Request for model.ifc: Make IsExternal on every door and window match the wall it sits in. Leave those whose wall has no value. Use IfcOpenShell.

First a look at what the model holds.

```python
import ifcopenshell
import ifcopenshell.util.element

model = ifcopenshell.open("model.ifc")
print(model.schema)
seen = {}
for e in model.by_type("IfcDoor") + model.by_type("IfcWindow"):
    if not e.FillsVoids:
        continue
    host = e.FillsVoids[0].RelatingOpeningElement.VoidsElements[0].RelatingBuildingElement
    own = ifcopenshell.util.element.get_pset(e, f"Pset_{e.is_a()[3:].removesuffix('StandardCase')}Common", "IsExternal")
    wall = ifcopenshell.util.element.get_pset(host, "Pset_WallCommon", "IsExternal")
    seen[e.is_a(), own, wall] = seen.get((e.is_a(), own, wall), 0) + 1
for (cls, own, wall), count in sorted(seen.items(), key=str):
    print(count, cls, "IsExternal:", own, "| host wall:", wall)
```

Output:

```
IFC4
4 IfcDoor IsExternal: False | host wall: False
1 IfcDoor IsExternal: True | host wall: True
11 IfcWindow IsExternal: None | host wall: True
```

```python
import ifcopenshell
import ifcopenshell.api.pset
import ifcopenshell.util.element

model = ifcopenshell.open("model.ifc")

count = 0
for ifc_class, pset_name in (("IfcDoor", "Pset_DoorCommon"), ("IfcWindow", "Pset_WindowCommon")):
    for e in model.by_type(ifc_class):
        if not e.FillsVoids:
            continue
        host = e.FillsVoids[0].RelatingOpeningElement.VoidsElements[0].RelatingBuildingElement
        external = ifcopenshell.util.element.get_pset(host, "Pset_WallCommon", "IsExternal")
        if external is None or ifcopenshell.util.element.get_pset(e, pset_name, "IsExternal") == external:
            continue
        pset = ifcopenshell.api.pset.add_pset(model, product=e, name=pset_name)
        ifcopenshell.api.pset.edit_pset(model, pset=pset, properties={"IsExternal": external})
        count += 1

print(count, "updated")

model.write("model_edited.ifc")
```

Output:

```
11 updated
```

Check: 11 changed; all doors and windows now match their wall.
